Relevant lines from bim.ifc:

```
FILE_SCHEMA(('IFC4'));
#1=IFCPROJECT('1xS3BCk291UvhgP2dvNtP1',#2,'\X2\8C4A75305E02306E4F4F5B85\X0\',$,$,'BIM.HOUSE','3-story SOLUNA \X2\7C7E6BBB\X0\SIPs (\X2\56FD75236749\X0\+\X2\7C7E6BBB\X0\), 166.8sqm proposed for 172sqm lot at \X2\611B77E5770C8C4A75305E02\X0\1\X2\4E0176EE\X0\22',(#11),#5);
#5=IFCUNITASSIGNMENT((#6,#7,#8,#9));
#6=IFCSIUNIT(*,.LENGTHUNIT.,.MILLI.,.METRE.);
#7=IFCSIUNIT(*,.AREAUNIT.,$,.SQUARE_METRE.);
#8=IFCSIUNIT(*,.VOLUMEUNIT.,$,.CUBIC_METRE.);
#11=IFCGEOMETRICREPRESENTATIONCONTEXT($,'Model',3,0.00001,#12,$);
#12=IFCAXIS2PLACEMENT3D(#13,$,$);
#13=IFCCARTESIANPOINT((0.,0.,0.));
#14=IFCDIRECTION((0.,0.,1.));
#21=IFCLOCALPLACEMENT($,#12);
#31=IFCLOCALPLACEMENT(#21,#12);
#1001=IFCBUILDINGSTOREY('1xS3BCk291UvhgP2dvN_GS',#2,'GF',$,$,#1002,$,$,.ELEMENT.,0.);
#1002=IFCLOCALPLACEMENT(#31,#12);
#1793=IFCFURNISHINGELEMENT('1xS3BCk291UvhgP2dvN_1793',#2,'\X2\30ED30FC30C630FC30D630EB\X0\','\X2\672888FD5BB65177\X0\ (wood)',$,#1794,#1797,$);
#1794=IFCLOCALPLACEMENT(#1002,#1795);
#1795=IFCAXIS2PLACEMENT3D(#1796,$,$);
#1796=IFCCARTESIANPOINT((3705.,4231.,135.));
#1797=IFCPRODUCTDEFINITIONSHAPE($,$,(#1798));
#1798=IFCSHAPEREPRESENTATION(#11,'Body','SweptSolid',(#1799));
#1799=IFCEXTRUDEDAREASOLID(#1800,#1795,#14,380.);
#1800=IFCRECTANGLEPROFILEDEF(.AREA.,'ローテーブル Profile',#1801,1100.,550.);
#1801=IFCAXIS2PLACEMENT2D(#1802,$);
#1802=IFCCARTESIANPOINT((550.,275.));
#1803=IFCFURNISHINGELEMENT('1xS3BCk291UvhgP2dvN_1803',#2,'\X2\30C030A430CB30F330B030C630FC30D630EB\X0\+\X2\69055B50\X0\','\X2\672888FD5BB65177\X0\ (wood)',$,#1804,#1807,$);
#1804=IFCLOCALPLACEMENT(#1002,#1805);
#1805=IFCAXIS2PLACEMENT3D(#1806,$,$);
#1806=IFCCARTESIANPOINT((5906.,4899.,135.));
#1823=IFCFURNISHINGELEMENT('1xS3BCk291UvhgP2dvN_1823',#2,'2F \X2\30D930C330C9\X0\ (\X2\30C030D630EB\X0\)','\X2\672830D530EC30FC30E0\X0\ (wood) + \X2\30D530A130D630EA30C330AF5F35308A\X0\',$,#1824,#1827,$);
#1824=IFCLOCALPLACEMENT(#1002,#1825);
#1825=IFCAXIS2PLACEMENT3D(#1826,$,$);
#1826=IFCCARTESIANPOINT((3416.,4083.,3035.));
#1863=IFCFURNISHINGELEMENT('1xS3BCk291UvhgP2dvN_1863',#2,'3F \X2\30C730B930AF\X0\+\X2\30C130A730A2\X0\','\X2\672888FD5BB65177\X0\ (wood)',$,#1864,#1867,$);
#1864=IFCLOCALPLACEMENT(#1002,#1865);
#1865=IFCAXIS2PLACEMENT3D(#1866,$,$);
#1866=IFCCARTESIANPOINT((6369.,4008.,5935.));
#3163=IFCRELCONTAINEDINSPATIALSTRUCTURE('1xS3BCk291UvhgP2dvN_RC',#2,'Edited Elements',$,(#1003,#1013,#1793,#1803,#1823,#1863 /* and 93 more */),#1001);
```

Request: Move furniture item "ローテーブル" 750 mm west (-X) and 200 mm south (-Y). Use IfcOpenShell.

```python
import ifcopenshell
import ifcopenshell.api.geometry
import ifcopenshell.util.placement

model = ifcopenshell.open("bim.ifc")

item = model.by_guid("1xS3BCk291UvhgP2dvN_1793")
matrix = ifcopenshell.util.placement.get_local_placement(item.ObjectPlacement)
matrix[0, 3] -= 750.0
matrix[1, 3] -= 200.0
ifcopenshell.api.geometry.edit_object_placement(model, product=item, matrix=matrix, is_si=False)

print(ifcopenshell.util.placement.get_local_placement(item.ObjectPlacement).round(3) + 0.0)

model.write("bim-out.ifc")
```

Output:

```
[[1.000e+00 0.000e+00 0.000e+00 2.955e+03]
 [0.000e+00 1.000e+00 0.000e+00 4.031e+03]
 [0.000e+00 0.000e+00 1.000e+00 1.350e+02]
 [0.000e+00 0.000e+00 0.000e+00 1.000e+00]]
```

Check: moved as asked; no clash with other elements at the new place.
